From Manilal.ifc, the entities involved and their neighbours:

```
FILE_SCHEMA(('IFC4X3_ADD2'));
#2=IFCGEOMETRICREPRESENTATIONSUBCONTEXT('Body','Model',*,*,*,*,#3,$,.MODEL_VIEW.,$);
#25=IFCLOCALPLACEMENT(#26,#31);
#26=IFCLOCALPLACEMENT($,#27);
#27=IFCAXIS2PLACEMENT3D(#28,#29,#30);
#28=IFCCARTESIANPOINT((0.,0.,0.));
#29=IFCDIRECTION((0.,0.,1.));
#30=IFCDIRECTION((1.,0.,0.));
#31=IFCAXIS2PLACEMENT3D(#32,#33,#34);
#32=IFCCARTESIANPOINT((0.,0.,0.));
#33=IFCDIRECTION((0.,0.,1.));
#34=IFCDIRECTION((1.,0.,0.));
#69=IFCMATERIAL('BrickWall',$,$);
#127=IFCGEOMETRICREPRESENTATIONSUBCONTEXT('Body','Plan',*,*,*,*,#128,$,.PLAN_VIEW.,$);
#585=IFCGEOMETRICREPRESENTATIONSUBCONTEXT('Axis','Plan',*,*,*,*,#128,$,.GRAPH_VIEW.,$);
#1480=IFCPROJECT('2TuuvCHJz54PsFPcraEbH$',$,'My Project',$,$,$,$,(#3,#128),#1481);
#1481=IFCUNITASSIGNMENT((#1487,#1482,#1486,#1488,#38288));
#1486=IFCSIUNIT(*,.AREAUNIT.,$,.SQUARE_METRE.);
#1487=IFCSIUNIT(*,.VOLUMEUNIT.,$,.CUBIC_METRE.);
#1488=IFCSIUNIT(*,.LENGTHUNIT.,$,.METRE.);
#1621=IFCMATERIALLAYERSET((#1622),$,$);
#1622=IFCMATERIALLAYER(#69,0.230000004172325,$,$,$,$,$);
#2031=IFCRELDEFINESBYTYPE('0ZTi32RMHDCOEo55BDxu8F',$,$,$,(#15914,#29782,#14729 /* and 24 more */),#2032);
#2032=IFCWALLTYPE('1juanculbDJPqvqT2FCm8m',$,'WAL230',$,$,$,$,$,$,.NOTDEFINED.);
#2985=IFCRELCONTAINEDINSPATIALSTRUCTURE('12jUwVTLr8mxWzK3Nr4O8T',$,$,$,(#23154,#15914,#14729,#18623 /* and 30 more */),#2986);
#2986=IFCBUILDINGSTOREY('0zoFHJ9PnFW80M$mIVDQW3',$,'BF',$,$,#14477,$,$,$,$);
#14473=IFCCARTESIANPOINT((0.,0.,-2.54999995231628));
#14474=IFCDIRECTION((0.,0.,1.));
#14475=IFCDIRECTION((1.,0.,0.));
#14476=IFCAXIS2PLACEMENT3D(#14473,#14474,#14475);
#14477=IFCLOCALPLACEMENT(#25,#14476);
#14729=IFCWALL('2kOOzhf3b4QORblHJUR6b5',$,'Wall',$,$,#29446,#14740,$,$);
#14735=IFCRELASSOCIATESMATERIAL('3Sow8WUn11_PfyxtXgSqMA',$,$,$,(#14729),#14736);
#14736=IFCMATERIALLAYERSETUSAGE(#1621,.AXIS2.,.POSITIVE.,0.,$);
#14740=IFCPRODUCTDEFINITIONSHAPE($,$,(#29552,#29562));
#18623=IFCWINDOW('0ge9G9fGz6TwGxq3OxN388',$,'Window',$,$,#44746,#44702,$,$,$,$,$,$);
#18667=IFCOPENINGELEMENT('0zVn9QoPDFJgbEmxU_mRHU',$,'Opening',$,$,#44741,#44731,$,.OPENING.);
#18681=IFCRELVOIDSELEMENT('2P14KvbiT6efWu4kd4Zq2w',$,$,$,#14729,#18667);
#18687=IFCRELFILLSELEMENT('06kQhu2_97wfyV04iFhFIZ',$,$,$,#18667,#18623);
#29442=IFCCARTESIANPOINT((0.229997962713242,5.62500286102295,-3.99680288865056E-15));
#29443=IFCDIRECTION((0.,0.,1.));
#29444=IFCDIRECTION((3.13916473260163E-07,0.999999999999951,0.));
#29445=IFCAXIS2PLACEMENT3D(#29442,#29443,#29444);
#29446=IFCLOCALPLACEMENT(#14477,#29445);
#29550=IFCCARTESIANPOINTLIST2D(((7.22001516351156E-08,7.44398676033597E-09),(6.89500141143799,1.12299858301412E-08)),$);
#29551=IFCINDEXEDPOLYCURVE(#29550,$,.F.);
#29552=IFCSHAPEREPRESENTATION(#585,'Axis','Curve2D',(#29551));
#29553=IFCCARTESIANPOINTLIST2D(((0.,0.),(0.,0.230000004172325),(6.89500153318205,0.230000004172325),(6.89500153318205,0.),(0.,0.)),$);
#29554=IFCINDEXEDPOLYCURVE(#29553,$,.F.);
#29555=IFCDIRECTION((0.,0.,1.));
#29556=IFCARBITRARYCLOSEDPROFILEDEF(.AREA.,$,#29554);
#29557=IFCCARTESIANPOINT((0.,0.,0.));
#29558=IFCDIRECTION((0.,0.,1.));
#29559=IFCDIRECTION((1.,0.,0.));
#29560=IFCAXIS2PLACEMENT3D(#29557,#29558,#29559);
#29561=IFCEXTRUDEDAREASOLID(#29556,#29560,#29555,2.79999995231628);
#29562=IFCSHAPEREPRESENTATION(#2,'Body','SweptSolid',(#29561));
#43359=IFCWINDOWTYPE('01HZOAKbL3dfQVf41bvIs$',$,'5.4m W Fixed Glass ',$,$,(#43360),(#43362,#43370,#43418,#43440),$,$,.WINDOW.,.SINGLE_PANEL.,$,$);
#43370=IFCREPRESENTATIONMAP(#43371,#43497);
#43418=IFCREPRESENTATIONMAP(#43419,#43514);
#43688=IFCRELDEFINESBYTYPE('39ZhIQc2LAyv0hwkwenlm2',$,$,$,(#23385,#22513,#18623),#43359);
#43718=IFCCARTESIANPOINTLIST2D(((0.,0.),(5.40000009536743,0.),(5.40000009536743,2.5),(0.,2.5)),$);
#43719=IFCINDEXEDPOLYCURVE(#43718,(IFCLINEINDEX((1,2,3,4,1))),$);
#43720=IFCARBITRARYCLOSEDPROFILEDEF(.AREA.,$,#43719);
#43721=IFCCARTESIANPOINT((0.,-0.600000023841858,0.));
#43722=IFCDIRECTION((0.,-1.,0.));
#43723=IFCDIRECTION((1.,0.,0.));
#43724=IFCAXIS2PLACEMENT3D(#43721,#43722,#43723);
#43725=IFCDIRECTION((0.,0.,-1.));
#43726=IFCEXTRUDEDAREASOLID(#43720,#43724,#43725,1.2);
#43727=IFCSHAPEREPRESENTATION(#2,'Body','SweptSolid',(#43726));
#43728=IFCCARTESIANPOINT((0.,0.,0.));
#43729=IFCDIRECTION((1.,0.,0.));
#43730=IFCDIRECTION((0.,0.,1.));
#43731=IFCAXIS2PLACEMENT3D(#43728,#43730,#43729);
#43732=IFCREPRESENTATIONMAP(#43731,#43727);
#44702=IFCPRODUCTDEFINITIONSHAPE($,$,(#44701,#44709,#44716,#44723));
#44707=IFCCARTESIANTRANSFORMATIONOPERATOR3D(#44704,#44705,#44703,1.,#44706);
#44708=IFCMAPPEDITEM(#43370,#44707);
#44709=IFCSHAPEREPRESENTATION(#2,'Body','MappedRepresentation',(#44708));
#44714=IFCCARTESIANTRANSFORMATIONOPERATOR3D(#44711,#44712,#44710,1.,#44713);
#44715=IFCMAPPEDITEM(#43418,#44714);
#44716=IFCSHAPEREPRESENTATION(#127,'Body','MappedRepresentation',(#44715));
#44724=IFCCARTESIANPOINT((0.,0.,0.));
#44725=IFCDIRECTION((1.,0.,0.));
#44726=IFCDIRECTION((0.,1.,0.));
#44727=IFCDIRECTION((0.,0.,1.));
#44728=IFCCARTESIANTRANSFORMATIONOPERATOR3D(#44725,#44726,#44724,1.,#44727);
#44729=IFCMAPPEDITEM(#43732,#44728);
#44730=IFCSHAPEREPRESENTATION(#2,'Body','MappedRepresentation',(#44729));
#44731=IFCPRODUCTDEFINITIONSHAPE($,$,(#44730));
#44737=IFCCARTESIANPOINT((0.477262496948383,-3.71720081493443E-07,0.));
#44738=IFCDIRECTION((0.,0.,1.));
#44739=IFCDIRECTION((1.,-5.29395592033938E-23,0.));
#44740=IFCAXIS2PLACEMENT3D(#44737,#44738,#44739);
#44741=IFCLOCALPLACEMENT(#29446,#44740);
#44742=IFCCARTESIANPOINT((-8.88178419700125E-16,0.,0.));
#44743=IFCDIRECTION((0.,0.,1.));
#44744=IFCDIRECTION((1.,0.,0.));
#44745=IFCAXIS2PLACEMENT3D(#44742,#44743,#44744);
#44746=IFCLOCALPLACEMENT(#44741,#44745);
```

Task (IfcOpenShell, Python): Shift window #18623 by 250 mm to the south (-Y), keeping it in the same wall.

```python
import ifcopenshell
import ifcopenshell.api.geometry
import ifcopenshell.util.placement

model = ifcopenshell.open("Manilal.ifc")

window = model.by_guid("0ge9G9fGz6TwGxq3OxN388")
opening = window.FillsVoids[0].RelatingOpeningElement
wall = opening.VoidsElements[0].RelatingBuildingElement

wall_matrix = ifcopenshell.util.placement.get_local_placement(wall.ObjectPlacement)
shift = wall_matrix[:3, 0] * -0.25
before = ifcopenshell.util.placement.get_local_placement(window.ObjectPlacement)[:3, 3].copy()

# The window is placed relative to its opening, so it follows when the opening moves.
matrix = ifcopenshell.util.placement.get_local_placement(opening.ObjectPlacement)
matrix[:3, 3] += shift
ifcopenshell.api.geometry.edit_object_placement(
    model, product=opening, matrix=matrix, is_si=False, should_transform_children=True
)

after = ifcopenshell.util.placement.get_local_placement(window.ObjectPlacement)[:3, 3]
print("window moved by", (after - before).round(3) + 0.0)

model.write("Manilal_v2.ifc")
```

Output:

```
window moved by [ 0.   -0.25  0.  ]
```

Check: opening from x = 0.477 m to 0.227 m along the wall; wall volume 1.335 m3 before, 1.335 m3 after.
